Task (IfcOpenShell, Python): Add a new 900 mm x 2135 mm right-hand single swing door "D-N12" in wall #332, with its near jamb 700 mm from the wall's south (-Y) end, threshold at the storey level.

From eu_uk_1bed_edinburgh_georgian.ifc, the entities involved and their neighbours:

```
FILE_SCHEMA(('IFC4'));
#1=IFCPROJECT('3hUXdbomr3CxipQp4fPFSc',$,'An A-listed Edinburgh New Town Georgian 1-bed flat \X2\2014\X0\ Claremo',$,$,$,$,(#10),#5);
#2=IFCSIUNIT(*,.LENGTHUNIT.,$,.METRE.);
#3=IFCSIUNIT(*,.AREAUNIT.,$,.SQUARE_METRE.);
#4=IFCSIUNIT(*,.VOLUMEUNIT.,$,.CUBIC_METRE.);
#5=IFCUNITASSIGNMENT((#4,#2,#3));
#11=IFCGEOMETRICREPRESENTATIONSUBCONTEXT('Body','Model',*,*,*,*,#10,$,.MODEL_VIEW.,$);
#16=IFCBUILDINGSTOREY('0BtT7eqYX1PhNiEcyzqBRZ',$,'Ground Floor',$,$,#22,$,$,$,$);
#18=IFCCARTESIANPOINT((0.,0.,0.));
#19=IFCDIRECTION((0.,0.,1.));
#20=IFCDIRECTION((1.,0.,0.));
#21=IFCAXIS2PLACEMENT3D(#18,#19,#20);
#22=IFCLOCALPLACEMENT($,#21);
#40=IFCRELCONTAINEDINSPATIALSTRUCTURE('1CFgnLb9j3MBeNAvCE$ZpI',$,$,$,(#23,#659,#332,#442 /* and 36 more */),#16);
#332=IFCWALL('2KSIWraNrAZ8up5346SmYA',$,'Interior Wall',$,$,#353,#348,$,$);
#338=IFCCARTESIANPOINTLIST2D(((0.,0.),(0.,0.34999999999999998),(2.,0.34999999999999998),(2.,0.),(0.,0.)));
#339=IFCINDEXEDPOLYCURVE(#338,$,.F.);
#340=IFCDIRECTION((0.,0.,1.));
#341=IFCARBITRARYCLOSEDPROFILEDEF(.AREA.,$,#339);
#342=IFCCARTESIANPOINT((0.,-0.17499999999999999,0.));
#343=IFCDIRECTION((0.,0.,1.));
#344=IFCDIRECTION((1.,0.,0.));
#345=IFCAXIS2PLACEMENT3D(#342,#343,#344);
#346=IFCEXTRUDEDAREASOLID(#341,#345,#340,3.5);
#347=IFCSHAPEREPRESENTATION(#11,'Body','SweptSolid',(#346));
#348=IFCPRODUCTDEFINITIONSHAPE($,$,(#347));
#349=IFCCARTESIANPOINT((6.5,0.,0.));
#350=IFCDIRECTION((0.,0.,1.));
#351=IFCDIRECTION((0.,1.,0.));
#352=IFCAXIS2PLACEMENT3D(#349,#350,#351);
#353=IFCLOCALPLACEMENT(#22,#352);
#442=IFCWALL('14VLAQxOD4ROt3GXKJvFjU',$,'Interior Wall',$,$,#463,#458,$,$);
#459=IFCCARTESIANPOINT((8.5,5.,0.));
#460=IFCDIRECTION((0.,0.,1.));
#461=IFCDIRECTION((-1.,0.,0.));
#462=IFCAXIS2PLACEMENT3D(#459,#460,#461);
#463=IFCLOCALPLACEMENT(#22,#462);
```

```python
import numpy as np
import ifcopenshell
import ifcopenshell.api.feature
import ifcopenshell.api.geometry
import ifcopenshell.api.root
import ifcopenshell.api.spatial
import ifcopenshell.geom
import ifcopenshell.util.element
import ifcopenshell.util.placement
import ifcopenshell.util.representation
import ifcopenshell.util.shape
import ifcopenshell.util.unit

model = ifcopenshell.open("eu_uk_1bed_edinburgh_georgian.ifc")
unit_scale = ifcopenshell.util.unit.calculate_unit_scale(model)
settings = ifcopenshell.geom.settings()


def volume(element):
    """Net volume in cubic metres, openings subtracted."""
    shape = ifcopenshell.geom.create_shape(settings, element)
    return ifcopenshell.util.shape.get_volume(shape.geometry)


wall = model.by_guid("2KSIWraNrAZ8up5346SmYA")
storey = ifcopenshell.util.element.get_container(wall, ifc_class="IfcBuildingStorey")
context = ifcopenshell.util.representation.get_context(model, "Model", "Body", "MODEL_VIEW")
before = volume(wall)

width, height, from_end, sill = 0.9, 2.135, 0.7, 0.0  # metres

# The wall runs along its own X axis, and the end named is its -X end.
wall_shape = ifcopenshell.geom.create_shape(settings, wall)
x, y, z = ifcopenshell.util.shape.get_vertices(wall_shape.geometry).T
start = x.min() + from_end
face, thickness = float(y.min()), float(y.max() - y.min())
wall_matrix = ifcopenshell.util.placement.get_local_placement(wall.ObjectPlacement)
level = ifcopenshell.util.placement.get_local_placement(storey.ObjectPlacement)[2, 3]


def in_wall(x, y):
    """Placement at x, y metres in the wall's axes, at sill height."""
    matrix = wall_matrix.copy()
    matrix[:, 3] = wall_matrix @ np.array([x / unit_scale, y / unit_scale, 0.0, 1.0])
    matrix[2, 3] = level + sill / unit_scale
    return matrix


# Opening: a box that overshoots both wall faces by 50 mm.
opening = ifcopenshell.api.root.create_entity(model, ifc_class="IfcOpeningElement", predefined_type="OPENING")
box = ifcopenshell.api.geometry.add_wall_representation(
    model, context=context, length=width, height=height, thickness=thickness + 0.1
)
ifcopenshell.api.geometry.assign_representation(model, product=opening, representation=box)
ifcopenshell.api.geometry.edit_object_placement(model, product=opening, matrix=in_wall(start, face - 0.05), is_si=False)
ifcopenshell.api.feature.add_feature(model, feature=opening, element=wall)

door = ifcopenshell.api.root.create_entity(model, ifc_class="IfcDoor", name="D-N12", predefined_type="DOOR")
door.OverallWidth, door.OverallHeight = width / unit_scale, height / unit_scale
door.OperationType = "SINGLE_SWING_RIGHT"
body = ifcopenshell.api.geometry.add_door_representation(
    model,
    context=context,
    overall_width=door.OverallWidth,
    overall_height=door.OverallHeight,
    operation_type="SINGLE_SWING_RIGHT",
    lining_properties={"LiningDepth": thickness / unit_scale, "ThresholdDepth": thickness / unit_scale},
)
ifcopenshell.api.geometry.assign_representation(model, product=door, representation=body)
ifcopenshell.api.spatial.assign_container(model, products=[door], relating_structure=storey)
ifcopenshell.api.feature.add_filling(model, opening=opening, element=door)

# The lining spans the wall, so the door starts at the wall face.
ifcopenshell.api.geometry.edit_object_placement(model, product=door, matrix=in_wall(start, face), is_si=False)

after = volume(wall)

print(f"wall volume {before:.3f} -> {after:.3f} m3")

model.write("eu_uk_1bed_edinburgh_georgian_v2.ifc")
```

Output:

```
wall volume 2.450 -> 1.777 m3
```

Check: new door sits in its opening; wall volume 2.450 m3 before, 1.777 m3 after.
